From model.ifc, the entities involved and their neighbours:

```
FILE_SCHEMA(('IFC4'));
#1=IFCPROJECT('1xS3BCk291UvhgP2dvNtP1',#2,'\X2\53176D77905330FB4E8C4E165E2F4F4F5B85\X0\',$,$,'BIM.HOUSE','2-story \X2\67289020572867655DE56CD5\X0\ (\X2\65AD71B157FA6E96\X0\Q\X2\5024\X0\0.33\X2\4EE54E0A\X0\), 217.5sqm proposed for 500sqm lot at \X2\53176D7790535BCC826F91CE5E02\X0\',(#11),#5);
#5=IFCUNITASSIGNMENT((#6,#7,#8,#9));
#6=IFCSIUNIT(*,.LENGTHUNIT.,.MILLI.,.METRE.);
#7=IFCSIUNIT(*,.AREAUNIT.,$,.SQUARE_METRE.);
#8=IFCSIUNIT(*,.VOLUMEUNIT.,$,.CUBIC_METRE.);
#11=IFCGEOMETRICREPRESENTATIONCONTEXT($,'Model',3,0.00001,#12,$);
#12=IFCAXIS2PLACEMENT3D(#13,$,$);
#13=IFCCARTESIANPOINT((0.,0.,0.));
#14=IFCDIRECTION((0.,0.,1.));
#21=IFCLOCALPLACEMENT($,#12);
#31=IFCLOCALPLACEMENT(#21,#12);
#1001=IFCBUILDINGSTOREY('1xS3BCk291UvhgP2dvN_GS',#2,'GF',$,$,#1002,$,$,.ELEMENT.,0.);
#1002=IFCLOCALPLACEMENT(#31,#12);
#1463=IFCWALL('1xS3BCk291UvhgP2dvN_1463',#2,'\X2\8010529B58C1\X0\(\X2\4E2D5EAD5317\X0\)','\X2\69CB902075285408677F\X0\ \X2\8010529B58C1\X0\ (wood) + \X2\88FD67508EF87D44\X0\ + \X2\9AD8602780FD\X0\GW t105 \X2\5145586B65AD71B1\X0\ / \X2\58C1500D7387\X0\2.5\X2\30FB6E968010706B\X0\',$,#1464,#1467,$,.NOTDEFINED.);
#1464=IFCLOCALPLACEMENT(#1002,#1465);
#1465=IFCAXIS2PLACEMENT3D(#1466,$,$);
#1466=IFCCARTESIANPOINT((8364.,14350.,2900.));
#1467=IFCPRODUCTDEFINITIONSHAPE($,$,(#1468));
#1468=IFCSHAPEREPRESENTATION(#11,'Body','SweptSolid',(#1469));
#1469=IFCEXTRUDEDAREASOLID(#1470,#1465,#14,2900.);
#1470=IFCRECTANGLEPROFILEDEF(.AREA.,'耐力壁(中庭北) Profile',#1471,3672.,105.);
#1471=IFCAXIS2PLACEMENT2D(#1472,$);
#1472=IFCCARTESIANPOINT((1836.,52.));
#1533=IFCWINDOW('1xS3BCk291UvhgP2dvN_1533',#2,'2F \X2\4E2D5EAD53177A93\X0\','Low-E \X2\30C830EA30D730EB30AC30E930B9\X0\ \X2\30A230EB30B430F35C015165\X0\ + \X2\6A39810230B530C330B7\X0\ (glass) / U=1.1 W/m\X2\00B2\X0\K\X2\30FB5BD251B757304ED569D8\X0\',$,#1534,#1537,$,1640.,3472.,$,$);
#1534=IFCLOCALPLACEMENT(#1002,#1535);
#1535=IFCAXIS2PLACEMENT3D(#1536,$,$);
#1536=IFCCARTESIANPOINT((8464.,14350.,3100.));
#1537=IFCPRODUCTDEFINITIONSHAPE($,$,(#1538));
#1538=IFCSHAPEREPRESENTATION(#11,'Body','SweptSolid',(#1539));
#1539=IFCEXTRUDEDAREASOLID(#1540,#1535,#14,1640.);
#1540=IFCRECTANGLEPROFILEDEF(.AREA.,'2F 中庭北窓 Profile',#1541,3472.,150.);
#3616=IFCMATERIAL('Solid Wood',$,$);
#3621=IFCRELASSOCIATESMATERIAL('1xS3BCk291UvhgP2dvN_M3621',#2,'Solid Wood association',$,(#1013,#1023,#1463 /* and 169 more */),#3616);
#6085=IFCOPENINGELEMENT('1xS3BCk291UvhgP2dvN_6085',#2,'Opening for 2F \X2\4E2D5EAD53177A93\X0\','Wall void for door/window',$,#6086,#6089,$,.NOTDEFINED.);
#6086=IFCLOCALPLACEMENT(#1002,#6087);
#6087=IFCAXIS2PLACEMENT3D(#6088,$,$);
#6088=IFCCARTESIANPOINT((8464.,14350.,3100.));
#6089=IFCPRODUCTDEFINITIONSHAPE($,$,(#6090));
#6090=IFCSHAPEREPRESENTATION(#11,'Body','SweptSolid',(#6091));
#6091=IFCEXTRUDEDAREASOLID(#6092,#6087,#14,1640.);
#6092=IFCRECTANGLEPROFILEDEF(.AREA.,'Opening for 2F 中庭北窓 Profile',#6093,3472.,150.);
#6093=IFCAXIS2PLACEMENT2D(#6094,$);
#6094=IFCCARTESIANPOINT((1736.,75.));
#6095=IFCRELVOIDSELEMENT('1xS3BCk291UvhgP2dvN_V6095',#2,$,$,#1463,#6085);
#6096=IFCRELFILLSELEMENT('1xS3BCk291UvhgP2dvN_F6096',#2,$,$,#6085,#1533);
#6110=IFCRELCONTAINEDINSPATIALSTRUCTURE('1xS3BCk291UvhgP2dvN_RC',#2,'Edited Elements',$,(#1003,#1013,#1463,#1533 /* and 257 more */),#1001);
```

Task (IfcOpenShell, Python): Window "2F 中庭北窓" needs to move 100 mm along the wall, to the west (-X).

```python
import ifcopenshell
import ifcopenshell.api.geometry
import ifcopenshell.util.placement
import ifcopenshell.util.unit

model = ifcopenshell.open("model.ifc")
unit_scale = ifcopenshell.util.unit.calculate_unit_scale(model)

window = model.by_guid("1xS3BCk291UvhgP2dvN_1533")
opening = window.FillsVoids[0].RelatingOpeningElement
wall = opening.VoidsElements[0].RelatingBuildingElement

wall_matrix = ifcopenshell.util.placement.get_local_placement(wall.ObjectPlacement)
shift = wall_matrix[:3, 0] * -0.1 / unit_scale
before = ifcopenshell.util.placement.get_local_placement(window.ObjectPlacement)[:3, 3].copy()

# The window is not placed relative to its opening, so move both.
for product in (opening, window):
    matrix = ifcopenshell.util.placement.get_local_placement(product.ObjectPlacement)
    matrix[:3, 3] += shift
    ifcopenshell.api.geometry.edit_object_placement(model, product=product, matrix=matrix, is_si=False)

after = ifcopenshell.util.placement.get_local_placement(window.ObjectPlacement)[:3, 3]
print("window moved by", (after - before).round(3) + 0.0)

model.write("model_v2.ifc")
```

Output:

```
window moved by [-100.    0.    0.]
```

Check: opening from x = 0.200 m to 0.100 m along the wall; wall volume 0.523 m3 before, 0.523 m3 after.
